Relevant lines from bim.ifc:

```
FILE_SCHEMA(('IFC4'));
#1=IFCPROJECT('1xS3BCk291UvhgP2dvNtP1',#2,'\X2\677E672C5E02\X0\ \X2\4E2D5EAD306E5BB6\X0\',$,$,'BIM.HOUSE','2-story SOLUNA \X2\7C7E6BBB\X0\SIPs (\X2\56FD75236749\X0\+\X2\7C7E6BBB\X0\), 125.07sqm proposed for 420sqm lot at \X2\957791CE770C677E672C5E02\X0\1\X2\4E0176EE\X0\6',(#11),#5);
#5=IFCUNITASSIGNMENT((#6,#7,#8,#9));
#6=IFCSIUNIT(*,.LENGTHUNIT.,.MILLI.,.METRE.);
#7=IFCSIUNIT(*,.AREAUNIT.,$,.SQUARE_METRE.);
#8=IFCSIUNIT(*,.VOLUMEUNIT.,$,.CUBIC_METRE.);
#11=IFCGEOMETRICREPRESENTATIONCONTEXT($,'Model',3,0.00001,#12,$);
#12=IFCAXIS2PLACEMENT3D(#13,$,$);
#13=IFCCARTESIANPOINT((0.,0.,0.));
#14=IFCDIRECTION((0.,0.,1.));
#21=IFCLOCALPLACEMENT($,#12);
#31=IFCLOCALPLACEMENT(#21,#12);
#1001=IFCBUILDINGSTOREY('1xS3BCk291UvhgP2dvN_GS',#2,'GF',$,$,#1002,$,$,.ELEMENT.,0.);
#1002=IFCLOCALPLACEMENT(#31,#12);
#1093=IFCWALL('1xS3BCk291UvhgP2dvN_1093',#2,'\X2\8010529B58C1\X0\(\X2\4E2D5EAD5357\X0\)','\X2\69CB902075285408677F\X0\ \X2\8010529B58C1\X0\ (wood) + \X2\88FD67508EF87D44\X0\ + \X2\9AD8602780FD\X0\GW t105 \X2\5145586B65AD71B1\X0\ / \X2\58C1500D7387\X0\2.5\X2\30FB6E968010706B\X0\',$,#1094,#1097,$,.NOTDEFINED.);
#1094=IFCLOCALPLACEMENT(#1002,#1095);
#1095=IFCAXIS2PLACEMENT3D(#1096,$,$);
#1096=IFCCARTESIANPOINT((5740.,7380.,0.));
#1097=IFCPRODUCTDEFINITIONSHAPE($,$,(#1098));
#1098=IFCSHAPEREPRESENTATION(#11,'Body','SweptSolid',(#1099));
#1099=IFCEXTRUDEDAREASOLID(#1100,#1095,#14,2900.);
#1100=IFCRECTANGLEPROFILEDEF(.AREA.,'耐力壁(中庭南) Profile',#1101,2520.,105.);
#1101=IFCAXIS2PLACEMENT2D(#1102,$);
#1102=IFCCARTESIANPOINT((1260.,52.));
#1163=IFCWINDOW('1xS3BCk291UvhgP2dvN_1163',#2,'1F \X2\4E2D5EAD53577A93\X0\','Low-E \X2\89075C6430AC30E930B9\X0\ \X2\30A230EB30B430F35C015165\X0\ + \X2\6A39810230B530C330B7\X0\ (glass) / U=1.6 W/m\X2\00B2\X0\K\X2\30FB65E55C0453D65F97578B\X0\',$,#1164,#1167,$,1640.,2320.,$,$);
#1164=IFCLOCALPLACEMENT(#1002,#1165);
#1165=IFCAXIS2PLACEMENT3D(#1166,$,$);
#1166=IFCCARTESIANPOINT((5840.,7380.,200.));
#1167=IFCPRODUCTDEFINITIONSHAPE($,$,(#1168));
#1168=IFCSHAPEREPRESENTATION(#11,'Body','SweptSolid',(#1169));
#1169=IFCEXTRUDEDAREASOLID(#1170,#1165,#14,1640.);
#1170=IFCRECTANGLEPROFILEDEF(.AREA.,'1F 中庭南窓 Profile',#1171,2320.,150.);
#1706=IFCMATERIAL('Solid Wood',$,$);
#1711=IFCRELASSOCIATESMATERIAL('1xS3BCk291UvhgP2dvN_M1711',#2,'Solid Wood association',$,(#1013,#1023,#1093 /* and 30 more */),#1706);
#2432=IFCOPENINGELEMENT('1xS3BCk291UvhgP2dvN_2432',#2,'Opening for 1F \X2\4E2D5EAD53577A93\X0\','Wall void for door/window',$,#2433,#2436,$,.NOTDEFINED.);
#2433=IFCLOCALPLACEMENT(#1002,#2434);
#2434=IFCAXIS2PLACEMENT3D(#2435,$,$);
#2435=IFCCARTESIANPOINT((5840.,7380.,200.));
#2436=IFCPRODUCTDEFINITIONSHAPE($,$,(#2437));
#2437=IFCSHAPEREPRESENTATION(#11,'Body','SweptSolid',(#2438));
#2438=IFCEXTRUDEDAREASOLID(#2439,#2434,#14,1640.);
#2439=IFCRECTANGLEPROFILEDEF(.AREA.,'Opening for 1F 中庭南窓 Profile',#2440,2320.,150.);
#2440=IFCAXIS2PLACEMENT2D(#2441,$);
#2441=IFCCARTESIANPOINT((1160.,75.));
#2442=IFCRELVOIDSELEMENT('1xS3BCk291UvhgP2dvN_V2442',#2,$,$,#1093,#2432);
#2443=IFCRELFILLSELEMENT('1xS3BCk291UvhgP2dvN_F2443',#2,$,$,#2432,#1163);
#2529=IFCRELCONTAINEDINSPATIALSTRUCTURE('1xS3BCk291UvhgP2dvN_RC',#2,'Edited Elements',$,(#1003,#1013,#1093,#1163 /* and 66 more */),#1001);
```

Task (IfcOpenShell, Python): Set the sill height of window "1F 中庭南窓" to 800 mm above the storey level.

```python
import numpy as np
import ifcopenshell
import ifcopenshell.api.geometry
import ifcopenshell.geom
import ifcopenshell.util.element
import ifcopenshell.util.placement
import ifcopenshell.util.shape
import ifcopenshell.util.unit

model = ifcopenshell.open("bim.ifc")
unit_scale = ifcopenshell.util.unit.calculate_unit_scale(model)

window = model.by_id(1163)
opening = window.FillsVoids[0].RelatingOpeningElement
storey = ifcopenshell.util.element.get_container(window, ifc_class="IfcBuildingStorey")
level = ifcopenshell.util.placement.get_local_placement(storey.ObjectPlacement)[2, 3]

# The opening's origin need not be at the sill, so measure its lowest point.
shape = ifcopenshell.geom.create_shape(ifcopenshell.geom.settings(), opening)
bottom = ifcopenshell.util.shape.get_shape_bottom_elevation(shape, shape.geometry) / unit_scale
dz = level + 800.0 - bottom

shift = np.array([0.0, 0.0, dz])
# The window is not placed relative to its opening, so move both.
for product in (opening, window):
    matrix = ifcopenshell.util.placement.get_local_placement(product.ObjectPlacement)
    matrix[:3, 3] += shift
    ifcopenshell.api.geometry.edit_object_placement(model, product=product, matrix=matrix, is_si=False)

print(f"moved by {dz * unit_scale:+.3f} m")

model.write("bim_updated.ifc")
```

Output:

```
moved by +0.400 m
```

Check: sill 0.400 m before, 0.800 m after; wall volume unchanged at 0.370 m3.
